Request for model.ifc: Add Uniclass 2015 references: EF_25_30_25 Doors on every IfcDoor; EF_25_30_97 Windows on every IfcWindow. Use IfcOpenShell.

First a look at what the model holds.

```python
import ifcopenshell

model = ifcopenshell.open("model.ifc")
print(model.schema)
print("classifications:", [c.Name for c in model.by_type("IfcClassification")])
for ifc_class in ("IfcDoor", "IfcRoof", "IfcStair", "IfcWall", "IfcWindow"):
    print(ifc_class, len(model.by_type(ifc_class)))
```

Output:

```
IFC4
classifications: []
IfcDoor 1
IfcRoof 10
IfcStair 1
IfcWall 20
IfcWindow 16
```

```python
import ifcopenshell
import ifcopenshell.api.classification

model = ifcopenshell.open("model.ifc")

system = ifcopenshell.api.classification.add_classification(model, classification="Uniclass 2015")

codes = {
    "IfcDoor": ("EF_25_30_25", "Doors"),
    "IfcWindow": ("EF_25_30_97", "Windows"),
}
for ifc_class, (code, name) in codes.items():
    products = model.by_type(ifc_class)
    ifcopenshell.api.classification.add_reference(
        model, products=products, classification=system, identification=code, name=name
    )
    print(code, len(products))

model.write("model_v2.ifc")
```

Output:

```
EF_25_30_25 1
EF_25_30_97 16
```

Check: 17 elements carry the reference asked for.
